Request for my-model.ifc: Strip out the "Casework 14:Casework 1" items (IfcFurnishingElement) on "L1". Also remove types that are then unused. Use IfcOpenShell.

First a look at what the model holds.

```python
import ifcopenshell
import ifcopenshell.util.element

model = ifcopenshell.open("my-model.ifc")
print(model.schema)
storey = next(s for s in model.by_type("IfcBuildingStorey") if s.Name == "L1")
furniture = [e for e in ifcopenshell.util.element.get_decomposition(storey) if e.is_a("IfcFurnishingElement")]
seen = {}
for e in furniture:
    element_type = ifcopenshell.util.element.get_type(e)
    name = element_type.Name if element_type not in (None, e) else None
    seen[name] = seen.get(name, 0) + 1
for name, count in sorted(seen.items(), key=str):
    print(count, "x", name)
```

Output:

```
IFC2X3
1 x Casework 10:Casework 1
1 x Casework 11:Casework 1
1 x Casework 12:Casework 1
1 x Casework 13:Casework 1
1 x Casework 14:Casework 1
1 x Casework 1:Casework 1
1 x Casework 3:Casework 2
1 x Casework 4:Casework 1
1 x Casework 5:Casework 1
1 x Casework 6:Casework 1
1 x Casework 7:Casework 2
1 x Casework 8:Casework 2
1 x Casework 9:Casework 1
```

```python
import ifcopenshell
import ifcopenshell.api.root
import ifcopenshell.util.element

model = ifcopenshell.open("my-model.ifc")

storey = next(s for s in model.by_type("IfcBuildingStorey") if s.Name == "L1")
furniture = [e for e in ifcopenshell.util.element.get_decomposition(storey) if e.is_a("IfcFurnishingElement")]
targets = [e for e in furniture if (t := ifcopenshell.util.element.get_type(e)) not in (None, e) and t.Name == "Casework 14:Casework 1"]
types = {ifcopenshell.util.element.get_type(e) for e in targets} - {None, *targets}

for e in targets:
    ifcopenshell.api.root.remove_product(model, product=e)
print(len(targets), "removed")

unused = [t for t in types if not ifcopenshell.util.element.get_types(t)]
for t in unused:
    ifcopenshell.api.root.remove_product(model, product=t)
print(len(unused), "unused types removed")

model.write("my-model_edited.ifc")
```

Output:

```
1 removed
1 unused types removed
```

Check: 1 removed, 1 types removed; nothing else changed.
